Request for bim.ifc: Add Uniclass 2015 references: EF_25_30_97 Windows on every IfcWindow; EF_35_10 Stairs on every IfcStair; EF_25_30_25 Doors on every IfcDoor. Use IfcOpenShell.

First a look at what the model holds.

```python
import ifcopenshell

model = ifcopenshell.open("bim.ifc")
print(model.schema)
print("classifications:", [c.Name for c in model.by_type("IfcClassification")])
for ifc_class in ("IfcDoor", "IfcRoof", "IfcStair", "IfcWall", "IfcWindow"):
    print(ifc_class, len(model.by_type(ifc_class)))
```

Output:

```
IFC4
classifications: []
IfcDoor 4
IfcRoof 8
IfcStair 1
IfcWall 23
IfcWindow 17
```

```python
import ifcopenshell
import ifcopenshell.api.classification

model = ifcopenshell.open("bim.ifc")

system = ifcopenshell.api.classification.add_classification(model, classification="Uniclass 2015")

codes = {
    "IfcWindow": ("EF_25_30_97", "Windows"),
    "IfcStair": ("EF_35_10", "Stairs"),
    "IfcDoor": ("EF_25_30_25", "Doors"),
}
for ifc_class, (code, name) in codes.items():
    products = model.by_type(ifc_class)
    ifcopenshell.api.classification.add_reference(
        model, products=products, classification=system, identification=code, name=name
    )
    print(code, len(products))

model.write("bim_edited.ifc")
```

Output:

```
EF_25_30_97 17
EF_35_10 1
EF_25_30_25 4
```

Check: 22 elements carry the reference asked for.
